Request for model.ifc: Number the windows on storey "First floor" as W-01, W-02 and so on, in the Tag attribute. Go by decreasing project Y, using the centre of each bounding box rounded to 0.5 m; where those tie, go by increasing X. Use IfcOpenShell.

First a look at what the model holds.

```python
import ifcopenshell
import ifcopenshell.util.element
import ifcopenshell.util.placement

model = ifcopenshell.open("model.ifc")
print(model.schema)
storey = next(s for s in model.by_type("IfcBuildingStorey") if s.Name == "First floor")
windows = [e for e in ifcopenshell.util.element.get_decomposition(storey) if e.is_a("IfcWindow")]
for e in sorted(windows, key=lambda e: e.id()):
    origin = ifcopenshell.util.placement.get_local_placement(e.ObjectPlacement)[:3, 3]
    print(e.id(), e.Tag, e.Name, origin.round(2) + 0.0, sep=" | ")
```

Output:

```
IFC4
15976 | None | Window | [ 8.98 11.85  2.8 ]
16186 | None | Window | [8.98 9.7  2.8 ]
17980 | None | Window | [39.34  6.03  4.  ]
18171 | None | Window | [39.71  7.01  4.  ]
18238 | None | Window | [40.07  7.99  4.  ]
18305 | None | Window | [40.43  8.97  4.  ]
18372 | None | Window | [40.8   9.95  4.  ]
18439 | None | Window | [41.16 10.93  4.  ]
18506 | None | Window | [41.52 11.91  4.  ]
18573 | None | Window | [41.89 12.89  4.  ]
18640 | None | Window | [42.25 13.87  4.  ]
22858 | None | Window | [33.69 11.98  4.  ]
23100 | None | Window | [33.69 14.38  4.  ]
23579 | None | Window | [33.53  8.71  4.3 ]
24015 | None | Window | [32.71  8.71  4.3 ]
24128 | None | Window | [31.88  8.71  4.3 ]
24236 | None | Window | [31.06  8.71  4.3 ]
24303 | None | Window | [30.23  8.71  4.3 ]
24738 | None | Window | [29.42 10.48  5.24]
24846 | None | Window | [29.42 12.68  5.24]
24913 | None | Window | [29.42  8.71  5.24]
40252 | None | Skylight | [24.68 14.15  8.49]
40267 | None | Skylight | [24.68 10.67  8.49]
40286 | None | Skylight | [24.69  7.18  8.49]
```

```python
import ifcopenshell
import ifcopenshell.geom
import ifcopenshell.util.element
import ifcopenshell.util.shape

model = ifcopenshell.open("model.ifc")
settings = ifcopenshell.geom.settings()
settings.set("use-world-coords", True)


def centre(element):
    shape = ifcopenshell.geom.create_shape(settings, element)
    return ifcopenshell.util.shape.get_bbox_centroid(shape.geometry)


storey = next(s for s in model.by_type("IfcBuildingStorey") if s.Name == "First floor")
windows = [e for e in ifcopenshell.util.element.get_decomposition(storey) if e.is_a("IfcWindow")]

# Insertion points can sit at a corner or the storey origin, so sort by the geometry (in metres).
centres = {e: centre(e) for e in windows}
windows.sort(key=lambda e: (-round(centres[e][1] / 0.5), centres[e][0]))

for i, e in enumerate(windows, start=1):
    number = f"W-{i:02d}"
    e.Tag = number
    print(e.id(), number)

model.write("model_v2.ifc")
```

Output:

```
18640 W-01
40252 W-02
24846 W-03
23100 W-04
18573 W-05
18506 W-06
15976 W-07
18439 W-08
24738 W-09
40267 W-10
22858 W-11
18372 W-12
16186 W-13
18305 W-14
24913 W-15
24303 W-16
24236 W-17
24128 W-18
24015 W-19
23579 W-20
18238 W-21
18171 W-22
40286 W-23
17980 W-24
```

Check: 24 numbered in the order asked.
